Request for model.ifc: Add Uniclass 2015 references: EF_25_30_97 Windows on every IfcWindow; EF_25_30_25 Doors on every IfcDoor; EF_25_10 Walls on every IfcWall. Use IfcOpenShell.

First a look at what the model holds.

```python
import ifcopenshell

model = ifcopenshell.open("model.ifc")
print(model.schema)
print("classifications:", [c.Name for c in model.by_type("IfcClassification")])
for ifc_class in ("IfcDoor", "IfcRoof", "IfcStair", "IfcWall", "IfcWindow"):
    print(ifc_class, len(model.by_type(ifc_class)))
```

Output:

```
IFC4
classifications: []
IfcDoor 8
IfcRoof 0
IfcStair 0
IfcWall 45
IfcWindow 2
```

```python
import ifcopenshell
import ifcopenshell.api.classification

model = ifcopenshell.open("model.ifc")

system = ifcopenshell.api.classification.add_classification(model, classification="Uniclass 2015")

codes = {
    "IfcWindow": ("EF_25_30_97", "Windows"),
    "IfcDoor": ("EF_25_30_25", "Doors"),
    "IfcWall": ("EF_25_10", "Walls"),
}
for ifc_class, (code, name) in codes.items():
    products = model.by_type(ifc_class)
    ifcopenshell.api.classification.add_reference(
        model, products=products, classification=system, identification=code, name=name
    )
    print(code, len(products))

model.write("model_v2.ifc")
```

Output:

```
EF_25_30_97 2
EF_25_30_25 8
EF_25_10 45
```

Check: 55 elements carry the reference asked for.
